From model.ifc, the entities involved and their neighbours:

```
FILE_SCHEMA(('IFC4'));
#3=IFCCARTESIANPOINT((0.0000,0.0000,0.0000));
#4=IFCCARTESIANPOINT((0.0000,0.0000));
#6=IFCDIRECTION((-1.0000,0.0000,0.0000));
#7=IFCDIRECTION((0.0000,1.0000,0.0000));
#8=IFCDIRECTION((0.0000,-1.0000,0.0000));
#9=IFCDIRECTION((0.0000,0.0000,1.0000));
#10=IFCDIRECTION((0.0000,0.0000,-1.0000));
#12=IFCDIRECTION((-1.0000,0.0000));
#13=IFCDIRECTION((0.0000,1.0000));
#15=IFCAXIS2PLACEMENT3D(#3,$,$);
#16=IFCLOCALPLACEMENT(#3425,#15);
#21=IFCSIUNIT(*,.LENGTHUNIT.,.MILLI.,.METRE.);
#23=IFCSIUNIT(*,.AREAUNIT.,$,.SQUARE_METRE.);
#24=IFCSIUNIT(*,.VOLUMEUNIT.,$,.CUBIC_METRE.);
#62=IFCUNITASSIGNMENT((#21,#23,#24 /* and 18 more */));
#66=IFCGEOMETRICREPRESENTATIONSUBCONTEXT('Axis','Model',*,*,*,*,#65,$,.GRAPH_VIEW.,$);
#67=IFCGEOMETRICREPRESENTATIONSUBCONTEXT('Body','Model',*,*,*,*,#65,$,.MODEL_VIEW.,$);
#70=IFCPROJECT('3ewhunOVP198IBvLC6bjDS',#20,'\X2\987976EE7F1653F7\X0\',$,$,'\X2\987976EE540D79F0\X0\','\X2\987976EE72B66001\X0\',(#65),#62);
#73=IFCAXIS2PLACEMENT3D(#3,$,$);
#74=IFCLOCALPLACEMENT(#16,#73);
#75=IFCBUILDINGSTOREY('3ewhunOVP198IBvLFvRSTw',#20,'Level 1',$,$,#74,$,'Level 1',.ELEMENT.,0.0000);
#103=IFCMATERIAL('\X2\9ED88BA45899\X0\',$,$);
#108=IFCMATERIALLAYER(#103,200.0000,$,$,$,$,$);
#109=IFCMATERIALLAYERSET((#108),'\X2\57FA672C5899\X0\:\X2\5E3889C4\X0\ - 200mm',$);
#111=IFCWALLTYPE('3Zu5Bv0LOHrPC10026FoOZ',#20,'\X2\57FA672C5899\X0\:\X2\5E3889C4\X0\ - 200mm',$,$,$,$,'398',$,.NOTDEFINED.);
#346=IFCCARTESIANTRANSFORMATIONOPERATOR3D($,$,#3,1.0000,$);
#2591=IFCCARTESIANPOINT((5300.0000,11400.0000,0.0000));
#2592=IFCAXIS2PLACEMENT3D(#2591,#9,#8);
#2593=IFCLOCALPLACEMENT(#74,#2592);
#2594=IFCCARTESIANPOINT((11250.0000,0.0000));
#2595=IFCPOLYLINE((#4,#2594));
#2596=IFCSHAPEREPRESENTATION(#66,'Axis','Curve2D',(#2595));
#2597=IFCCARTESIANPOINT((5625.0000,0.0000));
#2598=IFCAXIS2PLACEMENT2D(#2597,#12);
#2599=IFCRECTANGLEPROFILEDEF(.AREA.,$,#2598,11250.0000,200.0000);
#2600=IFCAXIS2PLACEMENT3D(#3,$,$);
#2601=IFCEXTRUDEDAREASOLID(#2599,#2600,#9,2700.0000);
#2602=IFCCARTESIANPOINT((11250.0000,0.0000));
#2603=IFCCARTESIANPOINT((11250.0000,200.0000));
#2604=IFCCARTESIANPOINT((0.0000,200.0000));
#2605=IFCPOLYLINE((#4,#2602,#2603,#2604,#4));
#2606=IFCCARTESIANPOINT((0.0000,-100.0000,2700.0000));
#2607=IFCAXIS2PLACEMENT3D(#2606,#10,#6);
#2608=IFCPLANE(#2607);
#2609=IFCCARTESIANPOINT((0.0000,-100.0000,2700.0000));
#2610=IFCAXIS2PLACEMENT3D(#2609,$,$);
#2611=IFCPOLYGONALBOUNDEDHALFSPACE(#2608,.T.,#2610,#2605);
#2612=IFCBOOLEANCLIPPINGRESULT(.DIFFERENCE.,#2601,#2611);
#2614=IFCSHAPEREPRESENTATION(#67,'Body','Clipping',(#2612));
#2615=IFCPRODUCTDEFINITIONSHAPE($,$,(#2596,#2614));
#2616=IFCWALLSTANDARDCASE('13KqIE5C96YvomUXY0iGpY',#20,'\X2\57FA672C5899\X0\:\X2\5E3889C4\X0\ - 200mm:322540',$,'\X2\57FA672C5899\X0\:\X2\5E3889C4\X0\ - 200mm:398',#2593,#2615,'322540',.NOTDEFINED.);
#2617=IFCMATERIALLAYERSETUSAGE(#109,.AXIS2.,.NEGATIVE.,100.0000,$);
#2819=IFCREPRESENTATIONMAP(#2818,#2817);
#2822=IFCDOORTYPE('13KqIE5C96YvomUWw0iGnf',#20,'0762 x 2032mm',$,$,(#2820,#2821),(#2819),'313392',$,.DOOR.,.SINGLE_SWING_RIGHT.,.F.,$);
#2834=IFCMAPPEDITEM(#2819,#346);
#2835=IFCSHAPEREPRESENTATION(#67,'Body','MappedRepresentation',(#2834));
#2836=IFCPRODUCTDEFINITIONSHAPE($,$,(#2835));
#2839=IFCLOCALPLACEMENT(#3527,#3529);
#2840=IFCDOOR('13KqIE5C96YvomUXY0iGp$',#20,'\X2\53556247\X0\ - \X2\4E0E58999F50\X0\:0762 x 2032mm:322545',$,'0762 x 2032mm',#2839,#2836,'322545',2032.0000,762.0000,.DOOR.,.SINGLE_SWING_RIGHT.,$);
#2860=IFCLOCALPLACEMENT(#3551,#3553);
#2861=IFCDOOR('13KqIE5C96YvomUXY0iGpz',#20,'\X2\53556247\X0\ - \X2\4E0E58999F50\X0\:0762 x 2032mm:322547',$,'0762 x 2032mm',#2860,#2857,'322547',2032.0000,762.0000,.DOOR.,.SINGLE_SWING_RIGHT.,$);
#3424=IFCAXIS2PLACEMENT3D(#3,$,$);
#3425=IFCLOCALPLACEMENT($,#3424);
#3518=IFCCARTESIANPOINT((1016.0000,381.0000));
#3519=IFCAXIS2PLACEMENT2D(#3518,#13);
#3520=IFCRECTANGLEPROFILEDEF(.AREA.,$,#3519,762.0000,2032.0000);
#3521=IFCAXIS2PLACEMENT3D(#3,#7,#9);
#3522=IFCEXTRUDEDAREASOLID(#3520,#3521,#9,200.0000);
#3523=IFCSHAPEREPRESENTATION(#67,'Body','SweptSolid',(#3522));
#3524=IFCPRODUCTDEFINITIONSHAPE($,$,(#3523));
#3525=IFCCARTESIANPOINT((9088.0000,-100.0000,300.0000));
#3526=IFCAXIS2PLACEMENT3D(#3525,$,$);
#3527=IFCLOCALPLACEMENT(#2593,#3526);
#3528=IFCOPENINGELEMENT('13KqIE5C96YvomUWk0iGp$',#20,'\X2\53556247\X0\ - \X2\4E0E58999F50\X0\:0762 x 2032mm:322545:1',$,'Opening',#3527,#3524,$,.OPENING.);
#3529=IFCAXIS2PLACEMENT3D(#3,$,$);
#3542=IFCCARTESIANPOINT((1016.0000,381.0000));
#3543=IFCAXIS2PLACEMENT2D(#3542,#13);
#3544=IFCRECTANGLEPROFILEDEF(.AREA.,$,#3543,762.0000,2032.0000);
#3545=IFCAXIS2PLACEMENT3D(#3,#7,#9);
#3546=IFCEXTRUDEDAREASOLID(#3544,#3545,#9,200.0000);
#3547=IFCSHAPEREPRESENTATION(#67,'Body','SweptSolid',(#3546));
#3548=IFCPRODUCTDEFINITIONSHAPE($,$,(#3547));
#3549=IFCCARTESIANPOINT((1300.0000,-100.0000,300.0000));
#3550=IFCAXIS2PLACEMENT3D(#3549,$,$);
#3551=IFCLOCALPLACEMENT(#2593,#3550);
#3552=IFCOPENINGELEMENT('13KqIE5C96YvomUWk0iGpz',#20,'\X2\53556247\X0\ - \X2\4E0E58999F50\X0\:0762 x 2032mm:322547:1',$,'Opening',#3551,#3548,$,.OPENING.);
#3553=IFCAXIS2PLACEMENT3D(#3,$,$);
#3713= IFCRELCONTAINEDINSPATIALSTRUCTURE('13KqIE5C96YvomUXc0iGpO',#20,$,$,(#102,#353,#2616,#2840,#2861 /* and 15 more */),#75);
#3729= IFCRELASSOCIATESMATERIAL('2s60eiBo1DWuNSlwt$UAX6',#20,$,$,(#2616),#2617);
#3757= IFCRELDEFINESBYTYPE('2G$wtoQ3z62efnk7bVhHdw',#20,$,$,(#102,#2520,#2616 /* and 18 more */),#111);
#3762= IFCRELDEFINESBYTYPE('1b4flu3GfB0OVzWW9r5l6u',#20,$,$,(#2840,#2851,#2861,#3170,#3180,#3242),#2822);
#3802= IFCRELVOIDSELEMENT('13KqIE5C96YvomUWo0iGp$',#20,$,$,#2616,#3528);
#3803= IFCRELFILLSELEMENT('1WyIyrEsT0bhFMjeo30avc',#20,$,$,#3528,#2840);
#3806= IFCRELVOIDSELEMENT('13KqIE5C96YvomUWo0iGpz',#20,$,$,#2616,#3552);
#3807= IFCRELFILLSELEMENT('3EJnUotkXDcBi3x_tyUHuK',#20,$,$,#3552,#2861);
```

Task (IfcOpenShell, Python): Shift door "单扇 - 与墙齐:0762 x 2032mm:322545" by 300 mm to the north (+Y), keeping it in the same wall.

```python
import ifcopenshell
import ifcopenshell.api.geometry
import ifcopenshell.util.placement
import ifcopenshell.util.unit

model = ifcopenshell.open("model.ifc")
unit_scale = ifcopenshell.util.unit.calculate_unit_scale(model)

door = model.by_guid("13KqIE5C96YvomUXY0iGp$")
opening = door.FillsVoids[0].RelatingOpeningElement
wall = opening.VoidsElements[0].RelatingBuildingElement

wall_matrix = ifcopenshell.util.placement.get_local_placement(wall.ObjectPlacement)
shift = wall_matrix[:3, 0] * -0.3 / unit_scale
before = ifcopenshell.util.placement.get_local_placement(door.ObjectPlacement)[:3, 3].copy()

# The door is placed relative to its opening, so it follows when the opening moves.
matrix = ifcopenshell.util.placement.get_local_placement(opening.ObjectPlacement)
matrix[:3, 3] += shift
ifcopenshell.api.geometry.edit_object_placement(
    model, product=opening, matrix=matrix, is_si=False, should_transform_children=True
)

after = ifcopenshell.util.placement.get_local_placement(door.ObjectPlacement)[:3, 3]
print("door moved by", (after - before).round(3) + 0.0)

model.write("model_edited.ifc")
```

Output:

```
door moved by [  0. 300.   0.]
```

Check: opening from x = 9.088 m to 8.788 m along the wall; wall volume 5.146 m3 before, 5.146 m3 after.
